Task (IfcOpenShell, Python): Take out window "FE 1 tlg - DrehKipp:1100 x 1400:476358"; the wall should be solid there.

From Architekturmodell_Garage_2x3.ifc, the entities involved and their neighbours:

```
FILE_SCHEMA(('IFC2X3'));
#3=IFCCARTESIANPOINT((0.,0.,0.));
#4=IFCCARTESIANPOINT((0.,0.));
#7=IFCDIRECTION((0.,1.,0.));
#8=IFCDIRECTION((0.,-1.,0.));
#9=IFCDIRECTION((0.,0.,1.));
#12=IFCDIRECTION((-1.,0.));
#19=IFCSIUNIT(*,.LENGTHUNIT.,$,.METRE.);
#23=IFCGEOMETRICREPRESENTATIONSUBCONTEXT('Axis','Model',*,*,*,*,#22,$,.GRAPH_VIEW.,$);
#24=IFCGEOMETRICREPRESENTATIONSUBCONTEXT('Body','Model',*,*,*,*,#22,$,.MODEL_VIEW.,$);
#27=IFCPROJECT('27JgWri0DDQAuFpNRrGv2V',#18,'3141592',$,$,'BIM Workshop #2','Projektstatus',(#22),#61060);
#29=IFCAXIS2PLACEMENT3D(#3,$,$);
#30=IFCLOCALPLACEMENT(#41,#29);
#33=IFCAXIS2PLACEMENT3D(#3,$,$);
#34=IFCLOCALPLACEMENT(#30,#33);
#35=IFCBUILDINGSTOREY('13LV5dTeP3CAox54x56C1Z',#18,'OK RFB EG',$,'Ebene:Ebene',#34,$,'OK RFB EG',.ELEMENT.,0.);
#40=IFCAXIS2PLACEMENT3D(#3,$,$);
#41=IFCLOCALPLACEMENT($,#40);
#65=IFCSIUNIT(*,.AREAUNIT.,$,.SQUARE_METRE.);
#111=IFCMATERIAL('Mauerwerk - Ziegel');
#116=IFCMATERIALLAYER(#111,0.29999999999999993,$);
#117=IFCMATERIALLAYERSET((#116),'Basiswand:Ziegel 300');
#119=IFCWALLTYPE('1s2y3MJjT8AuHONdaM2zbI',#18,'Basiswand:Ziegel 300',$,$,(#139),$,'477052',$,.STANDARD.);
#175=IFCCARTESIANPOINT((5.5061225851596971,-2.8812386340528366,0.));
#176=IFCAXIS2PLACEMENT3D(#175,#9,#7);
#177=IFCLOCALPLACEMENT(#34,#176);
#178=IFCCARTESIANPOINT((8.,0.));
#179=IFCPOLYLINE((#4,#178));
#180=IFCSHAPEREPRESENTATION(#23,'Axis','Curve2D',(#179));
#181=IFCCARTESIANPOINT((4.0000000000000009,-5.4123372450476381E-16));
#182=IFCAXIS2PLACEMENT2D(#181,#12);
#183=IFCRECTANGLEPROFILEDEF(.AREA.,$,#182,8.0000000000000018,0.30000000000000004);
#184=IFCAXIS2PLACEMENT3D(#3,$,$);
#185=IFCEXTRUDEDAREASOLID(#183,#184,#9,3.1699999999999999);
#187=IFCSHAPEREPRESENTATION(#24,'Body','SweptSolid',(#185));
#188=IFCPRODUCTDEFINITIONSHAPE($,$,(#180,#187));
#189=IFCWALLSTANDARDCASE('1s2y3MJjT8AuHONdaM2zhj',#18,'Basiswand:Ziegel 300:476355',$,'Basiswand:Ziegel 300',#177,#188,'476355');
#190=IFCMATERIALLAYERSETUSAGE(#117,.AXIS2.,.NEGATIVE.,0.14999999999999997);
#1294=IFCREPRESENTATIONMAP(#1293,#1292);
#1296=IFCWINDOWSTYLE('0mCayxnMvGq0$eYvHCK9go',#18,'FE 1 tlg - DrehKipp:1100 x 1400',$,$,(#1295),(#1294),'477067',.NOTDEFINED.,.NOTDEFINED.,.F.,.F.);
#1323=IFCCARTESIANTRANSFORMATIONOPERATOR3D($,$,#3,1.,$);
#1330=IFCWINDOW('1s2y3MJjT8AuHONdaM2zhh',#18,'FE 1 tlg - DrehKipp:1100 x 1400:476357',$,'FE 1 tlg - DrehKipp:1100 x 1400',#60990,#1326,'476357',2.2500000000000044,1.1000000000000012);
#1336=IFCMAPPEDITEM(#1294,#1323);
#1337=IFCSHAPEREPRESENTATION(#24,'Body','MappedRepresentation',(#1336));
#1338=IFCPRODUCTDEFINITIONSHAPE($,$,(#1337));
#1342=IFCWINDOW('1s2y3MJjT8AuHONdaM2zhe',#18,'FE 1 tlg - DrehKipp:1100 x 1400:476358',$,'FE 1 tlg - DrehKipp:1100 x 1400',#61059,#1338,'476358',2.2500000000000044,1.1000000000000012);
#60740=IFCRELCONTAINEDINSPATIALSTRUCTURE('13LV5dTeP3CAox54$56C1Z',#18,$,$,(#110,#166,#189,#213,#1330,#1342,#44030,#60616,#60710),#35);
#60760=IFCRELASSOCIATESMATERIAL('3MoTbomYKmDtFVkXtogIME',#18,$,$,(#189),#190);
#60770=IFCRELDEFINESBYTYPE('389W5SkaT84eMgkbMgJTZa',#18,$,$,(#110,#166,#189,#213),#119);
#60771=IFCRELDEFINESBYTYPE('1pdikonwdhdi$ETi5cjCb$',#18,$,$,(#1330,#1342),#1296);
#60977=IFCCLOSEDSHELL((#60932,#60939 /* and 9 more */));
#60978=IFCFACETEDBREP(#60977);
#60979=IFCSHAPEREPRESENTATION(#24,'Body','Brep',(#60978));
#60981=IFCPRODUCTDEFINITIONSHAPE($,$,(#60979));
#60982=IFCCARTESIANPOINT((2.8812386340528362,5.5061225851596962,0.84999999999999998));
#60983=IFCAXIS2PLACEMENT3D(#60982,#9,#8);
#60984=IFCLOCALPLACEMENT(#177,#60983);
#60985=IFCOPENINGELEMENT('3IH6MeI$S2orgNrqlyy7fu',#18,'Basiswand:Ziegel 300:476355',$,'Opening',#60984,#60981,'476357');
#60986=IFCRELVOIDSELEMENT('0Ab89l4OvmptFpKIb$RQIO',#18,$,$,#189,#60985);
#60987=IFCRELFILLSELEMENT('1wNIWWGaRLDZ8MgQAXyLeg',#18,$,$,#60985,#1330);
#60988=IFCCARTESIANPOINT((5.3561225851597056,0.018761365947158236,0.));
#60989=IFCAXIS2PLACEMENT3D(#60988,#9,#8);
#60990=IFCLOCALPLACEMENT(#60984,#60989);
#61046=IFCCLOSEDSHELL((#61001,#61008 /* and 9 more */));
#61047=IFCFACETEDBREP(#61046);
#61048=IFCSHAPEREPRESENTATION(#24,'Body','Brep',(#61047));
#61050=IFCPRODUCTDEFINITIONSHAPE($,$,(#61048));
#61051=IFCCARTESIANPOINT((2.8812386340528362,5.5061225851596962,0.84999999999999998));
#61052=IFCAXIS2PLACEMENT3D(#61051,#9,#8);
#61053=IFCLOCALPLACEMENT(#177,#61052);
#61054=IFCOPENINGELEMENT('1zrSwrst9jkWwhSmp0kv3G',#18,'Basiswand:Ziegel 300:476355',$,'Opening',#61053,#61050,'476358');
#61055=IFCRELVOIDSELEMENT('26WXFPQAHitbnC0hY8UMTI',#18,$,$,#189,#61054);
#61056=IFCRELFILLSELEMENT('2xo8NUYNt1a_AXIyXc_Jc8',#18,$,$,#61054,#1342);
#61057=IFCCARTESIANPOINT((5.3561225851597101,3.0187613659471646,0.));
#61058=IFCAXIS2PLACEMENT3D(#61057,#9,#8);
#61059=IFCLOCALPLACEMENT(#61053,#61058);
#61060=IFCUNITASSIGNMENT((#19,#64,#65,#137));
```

```python
import ifcopenshell
import ifcopenshell.api.feature
import ifcopenshell.api.root
import ifcopenshell.geom
import ifcopenshell.util.shape

model = ifcopenshell.open("Architekturmodell_Garage_2x3.ifc")
settings = ifcopenshell.geom.settings()


def volume(element):
    """Net volume in cubic metres, openings subtracted."""
    shape = ifcopenshell.geom.create_shape(settings, element)
    return ifcopenshell.util.shape.get_volume(shape.geometry)


window = model.by_id(1342)
opening = window.FillsVoids[0].RelatingOpeningElement
wall = opening.VoidsElements[0].RelatingBuildingElement
before = volume(wall)

ifcopenshell.api.root.remove_product(model, product=window)
ifcopenshell.api.feature.remove_feature(model, feature=opening)

after = volume(wall)

print(f"wall volume {before:.3f} -> {after:.3f} m3")

model.write("Architekturmodell_Garage_2x3_edited.ifc")
```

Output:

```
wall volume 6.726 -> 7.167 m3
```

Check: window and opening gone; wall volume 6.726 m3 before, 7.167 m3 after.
